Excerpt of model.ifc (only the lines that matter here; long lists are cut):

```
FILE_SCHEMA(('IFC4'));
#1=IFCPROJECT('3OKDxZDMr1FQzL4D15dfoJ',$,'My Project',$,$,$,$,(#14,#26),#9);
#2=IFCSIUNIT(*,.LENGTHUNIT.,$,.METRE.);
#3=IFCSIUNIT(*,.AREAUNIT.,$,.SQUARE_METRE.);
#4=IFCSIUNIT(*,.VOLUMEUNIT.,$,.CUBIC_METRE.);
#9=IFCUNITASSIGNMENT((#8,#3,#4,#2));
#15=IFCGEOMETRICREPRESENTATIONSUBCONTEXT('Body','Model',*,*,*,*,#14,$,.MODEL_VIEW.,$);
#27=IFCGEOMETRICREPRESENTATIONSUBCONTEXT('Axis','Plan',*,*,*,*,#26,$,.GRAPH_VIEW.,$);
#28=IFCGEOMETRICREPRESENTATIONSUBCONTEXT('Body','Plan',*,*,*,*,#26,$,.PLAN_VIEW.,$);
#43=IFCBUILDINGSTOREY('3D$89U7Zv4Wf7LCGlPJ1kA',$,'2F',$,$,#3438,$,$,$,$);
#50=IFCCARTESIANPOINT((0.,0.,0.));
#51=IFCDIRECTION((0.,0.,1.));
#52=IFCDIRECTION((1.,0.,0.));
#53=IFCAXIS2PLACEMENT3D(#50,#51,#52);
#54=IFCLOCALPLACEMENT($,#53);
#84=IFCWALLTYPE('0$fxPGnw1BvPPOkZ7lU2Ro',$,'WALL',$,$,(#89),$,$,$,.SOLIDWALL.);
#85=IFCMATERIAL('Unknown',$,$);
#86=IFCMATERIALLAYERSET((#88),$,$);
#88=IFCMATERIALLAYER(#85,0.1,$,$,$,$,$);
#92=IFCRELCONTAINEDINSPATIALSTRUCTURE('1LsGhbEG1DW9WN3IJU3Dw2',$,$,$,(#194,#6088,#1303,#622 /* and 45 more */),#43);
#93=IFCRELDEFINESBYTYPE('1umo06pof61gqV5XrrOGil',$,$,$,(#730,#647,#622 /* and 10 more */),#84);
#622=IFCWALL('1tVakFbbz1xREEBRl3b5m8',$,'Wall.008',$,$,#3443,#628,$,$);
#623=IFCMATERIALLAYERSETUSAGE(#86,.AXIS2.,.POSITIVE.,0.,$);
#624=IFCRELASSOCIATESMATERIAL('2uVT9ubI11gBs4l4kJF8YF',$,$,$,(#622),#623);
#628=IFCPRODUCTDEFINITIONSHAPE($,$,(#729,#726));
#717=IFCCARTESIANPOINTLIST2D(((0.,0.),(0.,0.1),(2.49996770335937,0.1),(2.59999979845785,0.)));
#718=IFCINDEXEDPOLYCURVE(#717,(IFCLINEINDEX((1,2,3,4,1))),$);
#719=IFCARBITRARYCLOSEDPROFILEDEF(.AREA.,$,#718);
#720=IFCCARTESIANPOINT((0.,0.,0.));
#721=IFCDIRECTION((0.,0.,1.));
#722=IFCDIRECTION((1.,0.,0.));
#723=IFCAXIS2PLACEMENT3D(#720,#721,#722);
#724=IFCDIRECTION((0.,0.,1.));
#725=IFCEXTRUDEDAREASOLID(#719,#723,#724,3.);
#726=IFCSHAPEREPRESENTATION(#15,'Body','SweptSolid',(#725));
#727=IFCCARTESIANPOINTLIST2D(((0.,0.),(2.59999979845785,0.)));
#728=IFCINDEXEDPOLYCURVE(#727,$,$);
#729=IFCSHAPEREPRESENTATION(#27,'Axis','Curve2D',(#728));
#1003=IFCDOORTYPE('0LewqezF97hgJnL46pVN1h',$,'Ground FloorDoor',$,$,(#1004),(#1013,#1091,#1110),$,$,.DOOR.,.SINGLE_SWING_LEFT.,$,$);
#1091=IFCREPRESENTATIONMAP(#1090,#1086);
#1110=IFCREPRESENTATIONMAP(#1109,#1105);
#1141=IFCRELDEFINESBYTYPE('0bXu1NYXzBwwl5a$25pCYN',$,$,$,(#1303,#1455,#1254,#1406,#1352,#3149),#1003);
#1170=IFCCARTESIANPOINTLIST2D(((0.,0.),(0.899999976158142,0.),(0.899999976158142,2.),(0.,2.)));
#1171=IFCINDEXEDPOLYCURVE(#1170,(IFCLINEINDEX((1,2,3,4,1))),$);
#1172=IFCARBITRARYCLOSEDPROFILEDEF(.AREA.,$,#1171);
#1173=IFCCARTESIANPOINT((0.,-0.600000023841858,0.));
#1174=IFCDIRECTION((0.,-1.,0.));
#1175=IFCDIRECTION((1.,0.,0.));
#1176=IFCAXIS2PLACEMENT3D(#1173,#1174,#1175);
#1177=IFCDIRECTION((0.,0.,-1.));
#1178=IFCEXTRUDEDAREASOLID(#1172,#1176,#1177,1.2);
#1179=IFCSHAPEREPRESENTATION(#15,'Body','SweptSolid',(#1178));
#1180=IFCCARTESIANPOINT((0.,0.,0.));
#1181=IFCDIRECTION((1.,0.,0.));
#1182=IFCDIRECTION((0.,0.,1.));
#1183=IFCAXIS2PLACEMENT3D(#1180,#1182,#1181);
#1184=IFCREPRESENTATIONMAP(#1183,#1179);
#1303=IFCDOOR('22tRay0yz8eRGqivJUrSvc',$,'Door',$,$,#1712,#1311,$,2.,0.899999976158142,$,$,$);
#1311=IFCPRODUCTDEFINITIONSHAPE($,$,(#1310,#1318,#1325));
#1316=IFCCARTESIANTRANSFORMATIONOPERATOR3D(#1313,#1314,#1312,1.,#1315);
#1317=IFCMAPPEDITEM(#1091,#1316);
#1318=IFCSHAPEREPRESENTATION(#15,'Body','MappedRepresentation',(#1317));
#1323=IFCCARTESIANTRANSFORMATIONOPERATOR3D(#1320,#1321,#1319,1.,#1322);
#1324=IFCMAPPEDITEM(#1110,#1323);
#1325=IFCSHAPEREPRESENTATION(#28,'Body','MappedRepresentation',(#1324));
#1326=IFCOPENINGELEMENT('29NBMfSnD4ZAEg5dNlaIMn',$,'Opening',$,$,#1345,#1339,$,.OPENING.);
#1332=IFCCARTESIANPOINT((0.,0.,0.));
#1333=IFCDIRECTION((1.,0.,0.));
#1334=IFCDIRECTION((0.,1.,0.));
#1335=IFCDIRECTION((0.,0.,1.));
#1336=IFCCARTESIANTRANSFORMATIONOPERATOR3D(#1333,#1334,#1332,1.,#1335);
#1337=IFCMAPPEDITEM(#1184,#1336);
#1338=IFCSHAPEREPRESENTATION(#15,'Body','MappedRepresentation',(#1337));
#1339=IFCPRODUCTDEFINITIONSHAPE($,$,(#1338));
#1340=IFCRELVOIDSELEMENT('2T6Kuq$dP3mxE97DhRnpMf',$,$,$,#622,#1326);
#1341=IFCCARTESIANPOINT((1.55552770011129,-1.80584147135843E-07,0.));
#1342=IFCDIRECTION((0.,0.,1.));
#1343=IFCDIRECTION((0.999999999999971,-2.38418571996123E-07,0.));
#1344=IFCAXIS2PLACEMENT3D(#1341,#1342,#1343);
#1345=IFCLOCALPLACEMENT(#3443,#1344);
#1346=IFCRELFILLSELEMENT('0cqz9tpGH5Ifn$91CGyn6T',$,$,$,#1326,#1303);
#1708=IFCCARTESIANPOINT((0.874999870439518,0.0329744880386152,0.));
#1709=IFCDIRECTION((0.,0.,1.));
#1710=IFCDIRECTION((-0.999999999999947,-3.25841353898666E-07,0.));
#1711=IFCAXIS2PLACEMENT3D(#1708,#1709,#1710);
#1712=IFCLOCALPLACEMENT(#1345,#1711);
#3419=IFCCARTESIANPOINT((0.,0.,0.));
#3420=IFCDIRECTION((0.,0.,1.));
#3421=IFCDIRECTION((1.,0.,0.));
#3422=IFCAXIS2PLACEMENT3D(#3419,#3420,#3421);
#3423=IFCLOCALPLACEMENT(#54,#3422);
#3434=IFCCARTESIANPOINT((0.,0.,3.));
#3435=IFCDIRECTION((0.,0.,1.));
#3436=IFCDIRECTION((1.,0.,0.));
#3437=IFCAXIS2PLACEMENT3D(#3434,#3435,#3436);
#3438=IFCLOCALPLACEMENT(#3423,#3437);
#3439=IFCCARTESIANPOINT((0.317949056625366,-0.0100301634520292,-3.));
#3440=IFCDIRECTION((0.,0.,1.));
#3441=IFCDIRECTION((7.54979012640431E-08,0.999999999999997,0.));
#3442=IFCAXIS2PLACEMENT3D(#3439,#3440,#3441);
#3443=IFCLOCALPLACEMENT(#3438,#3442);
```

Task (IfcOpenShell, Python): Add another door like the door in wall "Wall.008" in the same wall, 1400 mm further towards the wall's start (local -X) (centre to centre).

```python
import ifcopenshell
import ifcopenshell.api.feature
import ifcopenshell.api.geometry
import ifcopenshell.api.root
import ifcopenshell.geom
import ifcopenshell.util.element
import ifcopenshell.util.placement
import ifcopenshell.util.shape
import ifcopenshell.util.unit

model = ifcopenshell.open("model.ifc")
unit_scale = ifcopenshell.util.unit.calculate_unit_scale(model)
settings = ifcopenshell.geom.settings()


def volume(element):
    """Net volume in cubic metres, openings subtracted."""
    shape = ifcopenshell.geom.create_shape(settings, element)
    return ifcopenshell.util.shape.get_volume(shape.geometry)


door = model.by_id(1303)
opening = door.FillsVoids[0].RelatingOpeningElement
wall = opening.VoidsElements[0].RelatingBuildingElement
before = volume(wall)
shift = ifcopenshell.util.placement.get_local_placement(wall.ObjectPlacement)[:3, 0] * -1.4 / unit_scale

# copy_class copies the void relationship, type, container and properties, but no geometry.
new_opening = ifcopenshell.api.root.copy_class(model, product=opening)
new_opening.Representation = ifcopenshell.util.element.copy_deep(
    model, opening.Representation, exclude=["IfcGeometricRepresentationContext", "IfcRepresentationMap"]
)
new_door = ifcopenshell.api.root.copy_class(model, product=door)
new_door.Representation = ifcopenshell.util.element.copy_deep(
    model, door.Representation, exclude=["IfcGeometricRepresentationContext", "IfcRepresentationMap"]
)
ifcopenshell.api.feature.add_filling(model, opening=new_opening, element=new_door)

for old, new in ((opening, new_opening), (door, new_door)):
    matrix = ifcopenshell.util.placement.get_local_placement(old.ObjectPlacement)
    matrix[:3, 3] += shift
    ifcopenshell.api.geometry.edit_object_placement(model, product=new, matrix=matrix, is_si=False)

after = volume(wall)

print(f"wall volume {before:.3f} -> {after:.3f} m3")

model.write("model_v2.ifc")
```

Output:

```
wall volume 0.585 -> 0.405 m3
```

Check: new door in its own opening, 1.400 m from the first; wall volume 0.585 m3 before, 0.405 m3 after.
